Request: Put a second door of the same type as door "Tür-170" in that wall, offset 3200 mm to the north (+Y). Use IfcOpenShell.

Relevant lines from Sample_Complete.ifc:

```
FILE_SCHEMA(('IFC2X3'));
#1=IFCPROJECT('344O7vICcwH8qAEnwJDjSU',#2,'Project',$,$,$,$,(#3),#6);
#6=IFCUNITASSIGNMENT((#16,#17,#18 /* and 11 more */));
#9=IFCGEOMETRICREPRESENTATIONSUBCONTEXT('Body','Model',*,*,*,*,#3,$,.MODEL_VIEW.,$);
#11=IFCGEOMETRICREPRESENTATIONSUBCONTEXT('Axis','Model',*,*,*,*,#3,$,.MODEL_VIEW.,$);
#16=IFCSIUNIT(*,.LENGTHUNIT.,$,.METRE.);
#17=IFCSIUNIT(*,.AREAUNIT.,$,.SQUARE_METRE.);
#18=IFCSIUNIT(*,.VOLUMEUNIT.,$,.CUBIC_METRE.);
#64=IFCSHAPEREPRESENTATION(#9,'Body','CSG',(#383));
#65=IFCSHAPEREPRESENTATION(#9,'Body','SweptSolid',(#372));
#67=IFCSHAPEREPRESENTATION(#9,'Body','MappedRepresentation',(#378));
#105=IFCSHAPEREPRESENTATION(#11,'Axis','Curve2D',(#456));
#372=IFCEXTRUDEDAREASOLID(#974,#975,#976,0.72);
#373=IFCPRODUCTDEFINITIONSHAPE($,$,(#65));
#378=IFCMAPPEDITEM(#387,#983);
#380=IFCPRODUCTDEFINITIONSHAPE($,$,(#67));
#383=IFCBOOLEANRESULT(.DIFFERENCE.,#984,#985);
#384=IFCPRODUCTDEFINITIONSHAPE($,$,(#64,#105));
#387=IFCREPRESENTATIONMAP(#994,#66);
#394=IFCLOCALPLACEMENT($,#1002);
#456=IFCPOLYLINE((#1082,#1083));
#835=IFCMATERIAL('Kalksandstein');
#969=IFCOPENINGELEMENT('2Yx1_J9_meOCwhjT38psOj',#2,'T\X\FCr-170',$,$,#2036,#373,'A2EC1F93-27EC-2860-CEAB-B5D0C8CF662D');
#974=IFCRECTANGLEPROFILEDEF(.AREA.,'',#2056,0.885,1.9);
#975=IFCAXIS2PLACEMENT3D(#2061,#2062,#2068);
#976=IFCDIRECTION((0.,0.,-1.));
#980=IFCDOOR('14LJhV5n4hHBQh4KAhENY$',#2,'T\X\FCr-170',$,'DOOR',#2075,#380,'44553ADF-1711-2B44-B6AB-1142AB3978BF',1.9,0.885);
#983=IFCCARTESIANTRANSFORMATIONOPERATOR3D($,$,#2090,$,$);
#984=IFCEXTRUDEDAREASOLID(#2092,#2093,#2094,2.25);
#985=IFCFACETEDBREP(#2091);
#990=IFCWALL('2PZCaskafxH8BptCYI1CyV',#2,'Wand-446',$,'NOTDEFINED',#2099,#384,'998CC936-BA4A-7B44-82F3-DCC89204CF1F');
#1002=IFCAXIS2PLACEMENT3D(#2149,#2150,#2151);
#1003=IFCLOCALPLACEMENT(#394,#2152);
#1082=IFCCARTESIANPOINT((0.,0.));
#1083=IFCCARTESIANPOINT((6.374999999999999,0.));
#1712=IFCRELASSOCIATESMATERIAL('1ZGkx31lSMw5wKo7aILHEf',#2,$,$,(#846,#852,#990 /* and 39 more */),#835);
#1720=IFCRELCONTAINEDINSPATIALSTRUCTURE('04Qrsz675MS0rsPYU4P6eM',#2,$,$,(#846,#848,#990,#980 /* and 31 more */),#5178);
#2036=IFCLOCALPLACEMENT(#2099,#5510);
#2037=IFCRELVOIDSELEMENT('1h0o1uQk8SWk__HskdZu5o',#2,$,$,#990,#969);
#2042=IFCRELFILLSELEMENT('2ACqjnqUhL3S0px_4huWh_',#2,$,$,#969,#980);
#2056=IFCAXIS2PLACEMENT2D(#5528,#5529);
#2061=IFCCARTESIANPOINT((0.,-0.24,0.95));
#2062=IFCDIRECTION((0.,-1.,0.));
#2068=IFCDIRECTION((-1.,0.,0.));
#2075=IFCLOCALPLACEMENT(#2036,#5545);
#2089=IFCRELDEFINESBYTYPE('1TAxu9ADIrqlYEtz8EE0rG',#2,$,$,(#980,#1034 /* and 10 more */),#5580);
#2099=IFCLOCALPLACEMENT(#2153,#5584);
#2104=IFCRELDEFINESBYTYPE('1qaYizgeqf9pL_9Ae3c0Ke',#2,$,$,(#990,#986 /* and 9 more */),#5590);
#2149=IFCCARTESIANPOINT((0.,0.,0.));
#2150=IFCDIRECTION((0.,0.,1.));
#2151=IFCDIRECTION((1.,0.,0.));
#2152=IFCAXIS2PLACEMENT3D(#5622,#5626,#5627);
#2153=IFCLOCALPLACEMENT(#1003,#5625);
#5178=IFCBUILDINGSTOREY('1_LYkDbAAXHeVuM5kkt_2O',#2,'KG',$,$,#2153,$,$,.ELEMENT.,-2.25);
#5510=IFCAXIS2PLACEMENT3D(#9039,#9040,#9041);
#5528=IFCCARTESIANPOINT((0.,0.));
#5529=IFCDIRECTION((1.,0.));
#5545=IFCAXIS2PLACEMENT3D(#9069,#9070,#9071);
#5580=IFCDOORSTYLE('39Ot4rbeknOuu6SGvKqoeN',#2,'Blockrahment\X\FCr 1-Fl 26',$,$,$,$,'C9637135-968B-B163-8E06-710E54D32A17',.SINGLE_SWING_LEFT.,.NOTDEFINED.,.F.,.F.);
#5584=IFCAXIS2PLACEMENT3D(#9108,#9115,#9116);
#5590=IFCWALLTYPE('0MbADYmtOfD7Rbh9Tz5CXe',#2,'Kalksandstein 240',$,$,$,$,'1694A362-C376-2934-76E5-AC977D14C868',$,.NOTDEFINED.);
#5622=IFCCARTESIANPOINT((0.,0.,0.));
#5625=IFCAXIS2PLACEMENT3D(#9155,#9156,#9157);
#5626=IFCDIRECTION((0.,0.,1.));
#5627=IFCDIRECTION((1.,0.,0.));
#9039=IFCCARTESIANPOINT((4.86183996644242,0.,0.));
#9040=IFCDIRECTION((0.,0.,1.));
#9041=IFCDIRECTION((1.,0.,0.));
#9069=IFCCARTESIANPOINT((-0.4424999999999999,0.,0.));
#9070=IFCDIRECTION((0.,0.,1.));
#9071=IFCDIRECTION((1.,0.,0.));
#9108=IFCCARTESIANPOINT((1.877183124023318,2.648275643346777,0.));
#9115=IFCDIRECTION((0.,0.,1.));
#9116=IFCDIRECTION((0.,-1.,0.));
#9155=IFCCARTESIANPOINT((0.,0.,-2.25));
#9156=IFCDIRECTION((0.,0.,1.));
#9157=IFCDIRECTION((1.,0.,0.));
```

```python
import ifcopenshell
import ifcopenshell.api.feature
import ifcopenshell.api.geometry
import ifcopenshell.api.root
import ifcopenshell.geom
import ifcopenshell.util.element
import ifcopenshell.util.placement
import ifcopenshell.util.shape
import ifcopenshell.util.unit

model = ifcopenshell.open("Sample_Complete.ifc")
unit_scale = ifcopenshell.util.unit.calculate_unit_scale(model)
settings = ifcopenshell.geom.settings()


def volume(element):
    """Net volume in cubic metres, openings subtracted."""
    shape = ifcopenshell.geom.create_shape(settings, element)
    return ifcopenshell.util.shape.get_volume(shape.geometry)


def reuse_history(source, copy):
    """copy_class also copies each property set's owner history, people and application; keep the originals."""
    for rel in copy.IsDefinedBy:
        if rel.is_a("IfcRelDefinesByProperties") and (history := rel.RelatingPropertyDefinition.OwnerHistory):
            rel.RelatingPropertyDefinition.OwnerHistory = source.OwnerHistory
            ifcopenshell.util.element.remove_deep2(model, history)


door = model.by_guid("14LJhV5n4hHBQh4KAhENY$")
opening = door.FillsVoids[0].RelatingOpeningElement
wall = opening.VoidsElements[0].RelatingBuildingElement
before = volume(wall)
shift = ifcopenshell.util.placement.get_local_placement(wall.ObjectPlacement)[:3, 0] * -3.2 / unit_scale

# copy_class copies the void relationship, type, container and properties, but no geometry.
new_opening = ifcopenshell.api.root.copy_class(model, product=opening)
new_opening.Representation = ifcopenshell.util.element.copy_deep(
    model, opening.Representation, exclude=["IfcGeometricRepresentationContext", "IfcRepresentationMap"]
)
new_opening.Tag = None
new_door = ifcopenshell.api.root.copy_class(model, product=door)
new_door.Representation = ifcopenshell.util.element.copy_deep(
    model, door.Representation, exclude=["IfcGeometricRepresentationContext", "IfcRepresentationMap"]
)
new_door.Tag = None
reuse_history(door, new_door)
fills = ifcopenshell.api.feature.add_filling(model, opening=new_opening, element=new_door)
fills.OwnerHistory = new_door.OwnerHistory  # required in IFC2X3

for old, new in ((opening, new_opening), (door, new_door)):
    matrix = ifcopenshell.util.placement.get_local_placement(old.ObjectPlacement)
    matrix[:3, 3] += shift
    ifcopenshell.api.geometry.edit_object_placement(model, product=new, matrix=matrix, is_si=False)

after = volume(wall)

print(f"wall volume {before:.3f} -> {after:.3f} m3")

model.write("Sample_Complete_edited.ifc")
```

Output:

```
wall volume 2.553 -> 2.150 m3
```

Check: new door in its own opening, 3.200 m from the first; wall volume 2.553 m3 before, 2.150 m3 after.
